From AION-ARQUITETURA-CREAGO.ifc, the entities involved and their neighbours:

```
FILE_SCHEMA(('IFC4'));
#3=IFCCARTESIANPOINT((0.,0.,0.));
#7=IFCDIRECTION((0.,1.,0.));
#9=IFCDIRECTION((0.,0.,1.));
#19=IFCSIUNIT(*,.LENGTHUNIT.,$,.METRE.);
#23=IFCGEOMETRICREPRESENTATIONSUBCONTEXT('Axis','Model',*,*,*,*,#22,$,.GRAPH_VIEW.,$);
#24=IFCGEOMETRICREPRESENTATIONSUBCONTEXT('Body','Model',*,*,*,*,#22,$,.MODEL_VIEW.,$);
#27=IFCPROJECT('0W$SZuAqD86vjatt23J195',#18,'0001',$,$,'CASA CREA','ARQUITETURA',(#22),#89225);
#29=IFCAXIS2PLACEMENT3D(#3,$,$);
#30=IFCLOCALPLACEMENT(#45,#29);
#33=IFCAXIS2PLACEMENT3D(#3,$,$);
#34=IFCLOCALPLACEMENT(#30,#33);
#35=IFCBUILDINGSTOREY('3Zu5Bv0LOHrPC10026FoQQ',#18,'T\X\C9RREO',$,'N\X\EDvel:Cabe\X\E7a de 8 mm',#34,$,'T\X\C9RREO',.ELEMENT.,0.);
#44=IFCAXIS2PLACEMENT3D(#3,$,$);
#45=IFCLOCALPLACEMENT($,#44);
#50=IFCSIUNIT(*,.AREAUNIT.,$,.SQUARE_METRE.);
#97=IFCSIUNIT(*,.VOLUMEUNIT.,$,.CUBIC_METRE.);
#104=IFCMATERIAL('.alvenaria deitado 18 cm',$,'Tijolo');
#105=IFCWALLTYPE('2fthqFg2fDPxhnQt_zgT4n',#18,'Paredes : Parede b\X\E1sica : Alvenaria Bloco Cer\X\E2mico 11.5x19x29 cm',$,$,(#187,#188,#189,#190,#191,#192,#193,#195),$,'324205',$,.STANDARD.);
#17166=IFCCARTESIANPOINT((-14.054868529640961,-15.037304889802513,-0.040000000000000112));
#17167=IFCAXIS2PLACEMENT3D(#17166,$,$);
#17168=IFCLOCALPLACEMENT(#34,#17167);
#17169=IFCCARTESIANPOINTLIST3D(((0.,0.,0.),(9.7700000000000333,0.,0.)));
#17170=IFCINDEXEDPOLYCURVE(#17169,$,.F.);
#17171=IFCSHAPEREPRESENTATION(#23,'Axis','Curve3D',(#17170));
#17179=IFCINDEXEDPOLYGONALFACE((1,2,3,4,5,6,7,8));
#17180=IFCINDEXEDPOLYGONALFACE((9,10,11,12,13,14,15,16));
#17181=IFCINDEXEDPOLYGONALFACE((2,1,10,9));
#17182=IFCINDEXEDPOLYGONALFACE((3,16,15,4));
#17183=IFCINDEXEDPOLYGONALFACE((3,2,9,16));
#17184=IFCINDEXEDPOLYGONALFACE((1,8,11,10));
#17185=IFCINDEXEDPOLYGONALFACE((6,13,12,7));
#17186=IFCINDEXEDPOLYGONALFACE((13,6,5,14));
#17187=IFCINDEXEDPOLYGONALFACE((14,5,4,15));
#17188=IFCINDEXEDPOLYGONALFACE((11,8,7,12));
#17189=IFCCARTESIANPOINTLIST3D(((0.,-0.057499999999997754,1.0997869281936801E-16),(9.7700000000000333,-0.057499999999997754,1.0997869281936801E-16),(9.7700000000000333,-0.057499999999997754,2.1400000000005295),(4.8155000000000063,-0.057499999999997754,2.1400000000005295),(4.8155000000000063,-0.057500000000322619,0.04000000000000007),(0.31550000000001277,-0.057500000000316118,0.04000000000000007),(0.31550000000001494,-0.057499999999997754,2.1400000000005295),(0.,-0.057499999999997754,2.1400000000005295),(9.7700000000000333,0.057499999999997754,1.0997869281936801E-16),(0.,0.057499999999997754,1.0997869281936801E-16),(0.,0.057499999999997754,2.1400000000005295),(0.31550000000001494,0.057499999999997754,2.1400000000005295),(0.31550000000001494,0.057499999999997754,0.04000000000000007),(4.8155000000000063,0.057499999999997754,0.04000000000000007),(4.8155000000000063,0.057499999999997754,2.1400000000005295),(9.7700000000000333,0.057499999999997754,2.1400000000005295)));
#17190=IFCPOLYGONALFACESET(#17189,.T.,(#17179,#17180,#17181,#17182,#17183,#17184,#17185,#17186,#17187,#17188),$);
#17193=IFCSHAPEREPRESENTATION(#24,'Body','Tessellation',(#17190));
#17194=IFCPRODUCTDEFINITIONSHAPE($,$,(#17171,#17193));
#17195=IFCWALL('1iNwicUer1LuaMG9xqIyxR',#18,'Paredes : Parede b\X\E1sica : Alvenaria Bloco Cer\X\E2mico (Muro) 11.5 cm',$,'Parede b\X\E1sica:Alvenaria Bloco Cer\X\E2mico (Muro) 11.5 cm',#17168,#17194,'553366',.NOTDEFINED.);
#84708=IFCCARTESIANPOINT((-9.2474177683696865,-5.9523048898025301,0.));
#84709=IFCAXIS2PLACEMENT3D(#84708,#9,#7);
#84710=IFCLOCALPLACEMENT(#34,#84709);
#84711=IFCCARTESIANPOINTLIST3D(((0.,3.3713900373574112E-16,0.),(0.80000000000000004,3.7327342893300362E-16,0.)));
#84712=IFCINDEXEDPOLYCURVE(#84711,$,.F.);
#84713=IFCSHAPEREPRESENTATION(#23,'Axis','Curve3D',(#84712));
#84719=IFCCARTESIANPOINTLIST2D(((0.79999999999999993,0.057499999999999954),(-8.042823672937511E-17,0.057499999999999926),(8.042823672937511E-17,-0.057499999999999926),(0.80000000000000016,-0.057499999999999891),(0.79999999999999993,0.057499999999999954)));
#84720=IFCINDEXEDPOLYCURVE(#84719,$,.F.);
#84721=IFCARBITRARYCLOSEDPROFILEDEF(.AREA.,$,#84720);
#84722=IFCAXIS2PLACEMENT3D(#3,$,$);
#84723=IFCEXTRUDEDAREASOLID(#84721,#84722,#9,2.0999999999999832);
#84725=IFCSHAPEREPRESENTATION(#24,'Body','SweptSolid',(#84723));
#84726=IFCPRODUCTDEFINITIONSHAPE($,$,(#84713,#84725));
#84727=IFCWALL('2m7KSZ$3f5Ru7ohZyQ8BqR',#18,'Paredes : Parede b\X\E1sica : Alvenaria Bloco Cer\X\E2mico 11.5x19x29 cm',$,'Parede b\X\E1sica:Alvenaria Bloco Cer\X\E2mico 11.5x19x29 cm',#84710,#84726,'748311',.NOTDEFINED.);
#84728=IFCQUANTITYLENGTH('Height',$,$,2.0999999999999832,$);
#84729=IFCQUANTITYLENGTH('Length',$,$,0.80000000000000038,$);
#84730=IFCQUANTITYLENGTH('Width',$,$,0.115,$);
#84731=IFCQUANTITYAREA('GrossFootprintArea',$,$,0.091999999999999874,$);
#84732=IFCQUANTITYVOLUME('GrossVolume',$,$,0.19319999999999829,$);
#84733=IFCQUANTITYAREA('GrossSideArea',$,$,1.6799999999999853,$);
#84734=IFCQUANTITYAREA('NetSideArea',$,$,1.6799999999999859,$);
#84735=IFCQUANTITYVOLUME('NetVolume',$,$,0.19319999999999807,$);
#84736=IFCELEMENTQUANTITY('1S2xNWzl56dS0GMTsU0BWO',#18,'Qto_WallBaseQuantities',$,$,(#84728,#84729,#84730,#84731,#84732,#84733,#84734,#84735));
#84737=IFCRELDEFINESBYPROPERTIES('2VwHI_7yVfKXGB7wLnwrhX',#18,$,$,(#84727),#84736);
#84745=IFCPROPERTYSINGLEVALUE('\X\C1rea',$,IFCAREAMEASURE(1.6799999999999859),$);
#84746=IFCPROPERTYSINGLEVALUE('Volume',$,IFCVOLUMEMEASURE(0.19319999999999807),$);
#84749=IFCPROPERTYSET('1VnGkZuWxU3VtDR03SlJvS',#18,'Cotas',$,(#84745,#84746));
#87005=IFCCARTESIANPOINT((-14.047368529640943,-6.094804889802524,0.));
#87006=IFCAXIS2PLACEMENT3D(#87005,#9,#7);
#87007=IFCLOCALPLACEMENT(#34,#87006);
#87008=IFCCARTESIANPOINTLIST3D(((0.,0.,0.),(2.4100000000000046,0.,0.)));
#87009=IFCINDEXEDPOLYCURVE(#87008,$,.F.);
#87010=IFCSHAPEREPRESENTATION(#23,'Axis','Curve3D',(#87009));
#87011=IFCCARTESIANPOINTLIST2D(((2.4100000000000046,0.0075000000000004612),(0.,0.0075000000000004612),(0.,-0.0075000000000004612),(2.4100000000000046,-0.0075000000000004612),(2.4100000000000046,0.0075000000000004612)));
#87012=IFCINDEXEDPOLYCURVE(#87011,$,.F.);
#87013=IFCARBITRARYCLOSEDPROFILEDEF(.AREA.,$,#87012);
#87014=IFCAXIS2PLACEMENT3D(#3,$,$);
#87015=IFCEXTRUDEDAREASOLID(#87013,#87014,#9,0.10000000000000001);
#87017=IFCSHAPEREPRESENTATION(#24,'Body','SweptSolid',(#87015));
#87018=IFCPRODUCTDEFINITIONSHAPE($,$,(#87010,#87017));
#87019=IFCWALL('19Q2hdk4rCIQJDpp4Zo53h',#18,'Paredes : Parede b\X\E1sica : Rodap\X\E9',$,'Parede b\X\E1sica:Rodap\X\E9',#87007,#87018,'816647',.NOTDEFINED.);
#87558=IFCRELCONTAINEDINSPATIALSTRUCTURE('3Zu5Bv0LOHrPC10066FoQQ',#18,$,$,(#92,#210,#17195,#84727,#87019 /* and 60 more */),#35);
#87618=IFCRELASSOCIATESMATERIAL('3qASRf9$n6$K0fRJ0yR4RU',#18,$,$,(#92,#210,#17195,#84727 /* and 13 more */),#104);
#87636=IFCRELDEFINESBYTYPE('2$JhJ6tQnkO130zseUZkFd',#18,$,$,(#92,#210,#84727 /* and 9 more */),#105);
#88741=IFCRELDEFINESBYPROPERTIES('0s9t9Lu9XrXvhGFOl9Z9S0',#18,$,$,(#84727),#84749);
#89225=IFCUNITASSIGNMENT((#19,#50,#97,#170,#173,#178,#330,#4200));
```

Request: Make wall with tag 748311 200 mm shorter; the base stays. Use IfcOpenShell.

```python
import ifcopenshell
import ifcopenshell.api.pset
import ifcopenshell.geom
import ifcopenshell.util.element
import ifcopenshell.util.representation
import ifcopenshell.util.shape
import ifcopenshell.util.unit

model = ifcopenshell.open("AION-ARQUITETURA-CREAGO.ifc")
unit_scale = ifcopenshell.util.unit.calculate_unit_scale(model)
area_scale = ifcopenshell.util.unit.calculate_unit_scale(model, "AREAUNIT")
volume_scale = ifcopenshell.util.unit.calculate_unit_scale(model, "VOLUMEUNIT")
settings = ifcopenshell.geom.settings()


def volume(element):
    """Net volume in cubic metres, openings subtracted."""
    shape = ifcopenshell.geom.create_shape(settings, element)
    return ifcopenshell.util.shape.get_volume(shape.geometry)


wall = model.by_guid("2m7KSZ$3f5Ru7ohZyQ8BqR")
before = volume(wall)

body = ifcopenshell.util.representation.get_representation(wall, "Model", "Body")
solid = body.Items[0]
old_height = solid.Depth
solid.Depth -= 0.2
after = volume(wall)
thickness = 0.115  # wall thickness in metres

# Update the stored height, areas and volumes.
qto = model.by_id(ifcopenshell.util.element.get_pset(wall, "Qto_WallBaseQuantities", should_inherit=False)["id"])
ifcopenshell.api.pset.edit_qto(model, qto=qto, properties={
    "Height": solid.Depth,
    "GrossVolume": ifcopenshell.util.element.get_pset(wall, "Qto_WallBaseQuantities", "GrossVolume") * solid.Depth / old_height,
    "GrossSideArea": ifcopenshell.util.element.get_pset(wall, "Qto_WallBaseQuantities", "GrossSideArea") * solid.Depth / old_height,
    "NetSideArea": after / thickness / area_scale,
    "NetVolume": after / volume_scale,
})
pset = model.by_id(ifcopenshell.util.element.get_pset(wall, "Cotas", should_inherit=False)["id"])
ifcopenshell.api.pset.edit_pset(model, pset=pset, properties={
    "Área": model.create_entity("IfcAreaMeasure", after / thickness / area_scale),
    "Volume": model.create_entity("IfcVolumeMeasure", after / volume_scale),
})

print(f"height {old_height:g} -> {solid.Depth:g}, volume {before:.3f} -> {after:.3f} m3")

model.write("AION-ARQUITETURA-CREAGO_edited.ifc")
```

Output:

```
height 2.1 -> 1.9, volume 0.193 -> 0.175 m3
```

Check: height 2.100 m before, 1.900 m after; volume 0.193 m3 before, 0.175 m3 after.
